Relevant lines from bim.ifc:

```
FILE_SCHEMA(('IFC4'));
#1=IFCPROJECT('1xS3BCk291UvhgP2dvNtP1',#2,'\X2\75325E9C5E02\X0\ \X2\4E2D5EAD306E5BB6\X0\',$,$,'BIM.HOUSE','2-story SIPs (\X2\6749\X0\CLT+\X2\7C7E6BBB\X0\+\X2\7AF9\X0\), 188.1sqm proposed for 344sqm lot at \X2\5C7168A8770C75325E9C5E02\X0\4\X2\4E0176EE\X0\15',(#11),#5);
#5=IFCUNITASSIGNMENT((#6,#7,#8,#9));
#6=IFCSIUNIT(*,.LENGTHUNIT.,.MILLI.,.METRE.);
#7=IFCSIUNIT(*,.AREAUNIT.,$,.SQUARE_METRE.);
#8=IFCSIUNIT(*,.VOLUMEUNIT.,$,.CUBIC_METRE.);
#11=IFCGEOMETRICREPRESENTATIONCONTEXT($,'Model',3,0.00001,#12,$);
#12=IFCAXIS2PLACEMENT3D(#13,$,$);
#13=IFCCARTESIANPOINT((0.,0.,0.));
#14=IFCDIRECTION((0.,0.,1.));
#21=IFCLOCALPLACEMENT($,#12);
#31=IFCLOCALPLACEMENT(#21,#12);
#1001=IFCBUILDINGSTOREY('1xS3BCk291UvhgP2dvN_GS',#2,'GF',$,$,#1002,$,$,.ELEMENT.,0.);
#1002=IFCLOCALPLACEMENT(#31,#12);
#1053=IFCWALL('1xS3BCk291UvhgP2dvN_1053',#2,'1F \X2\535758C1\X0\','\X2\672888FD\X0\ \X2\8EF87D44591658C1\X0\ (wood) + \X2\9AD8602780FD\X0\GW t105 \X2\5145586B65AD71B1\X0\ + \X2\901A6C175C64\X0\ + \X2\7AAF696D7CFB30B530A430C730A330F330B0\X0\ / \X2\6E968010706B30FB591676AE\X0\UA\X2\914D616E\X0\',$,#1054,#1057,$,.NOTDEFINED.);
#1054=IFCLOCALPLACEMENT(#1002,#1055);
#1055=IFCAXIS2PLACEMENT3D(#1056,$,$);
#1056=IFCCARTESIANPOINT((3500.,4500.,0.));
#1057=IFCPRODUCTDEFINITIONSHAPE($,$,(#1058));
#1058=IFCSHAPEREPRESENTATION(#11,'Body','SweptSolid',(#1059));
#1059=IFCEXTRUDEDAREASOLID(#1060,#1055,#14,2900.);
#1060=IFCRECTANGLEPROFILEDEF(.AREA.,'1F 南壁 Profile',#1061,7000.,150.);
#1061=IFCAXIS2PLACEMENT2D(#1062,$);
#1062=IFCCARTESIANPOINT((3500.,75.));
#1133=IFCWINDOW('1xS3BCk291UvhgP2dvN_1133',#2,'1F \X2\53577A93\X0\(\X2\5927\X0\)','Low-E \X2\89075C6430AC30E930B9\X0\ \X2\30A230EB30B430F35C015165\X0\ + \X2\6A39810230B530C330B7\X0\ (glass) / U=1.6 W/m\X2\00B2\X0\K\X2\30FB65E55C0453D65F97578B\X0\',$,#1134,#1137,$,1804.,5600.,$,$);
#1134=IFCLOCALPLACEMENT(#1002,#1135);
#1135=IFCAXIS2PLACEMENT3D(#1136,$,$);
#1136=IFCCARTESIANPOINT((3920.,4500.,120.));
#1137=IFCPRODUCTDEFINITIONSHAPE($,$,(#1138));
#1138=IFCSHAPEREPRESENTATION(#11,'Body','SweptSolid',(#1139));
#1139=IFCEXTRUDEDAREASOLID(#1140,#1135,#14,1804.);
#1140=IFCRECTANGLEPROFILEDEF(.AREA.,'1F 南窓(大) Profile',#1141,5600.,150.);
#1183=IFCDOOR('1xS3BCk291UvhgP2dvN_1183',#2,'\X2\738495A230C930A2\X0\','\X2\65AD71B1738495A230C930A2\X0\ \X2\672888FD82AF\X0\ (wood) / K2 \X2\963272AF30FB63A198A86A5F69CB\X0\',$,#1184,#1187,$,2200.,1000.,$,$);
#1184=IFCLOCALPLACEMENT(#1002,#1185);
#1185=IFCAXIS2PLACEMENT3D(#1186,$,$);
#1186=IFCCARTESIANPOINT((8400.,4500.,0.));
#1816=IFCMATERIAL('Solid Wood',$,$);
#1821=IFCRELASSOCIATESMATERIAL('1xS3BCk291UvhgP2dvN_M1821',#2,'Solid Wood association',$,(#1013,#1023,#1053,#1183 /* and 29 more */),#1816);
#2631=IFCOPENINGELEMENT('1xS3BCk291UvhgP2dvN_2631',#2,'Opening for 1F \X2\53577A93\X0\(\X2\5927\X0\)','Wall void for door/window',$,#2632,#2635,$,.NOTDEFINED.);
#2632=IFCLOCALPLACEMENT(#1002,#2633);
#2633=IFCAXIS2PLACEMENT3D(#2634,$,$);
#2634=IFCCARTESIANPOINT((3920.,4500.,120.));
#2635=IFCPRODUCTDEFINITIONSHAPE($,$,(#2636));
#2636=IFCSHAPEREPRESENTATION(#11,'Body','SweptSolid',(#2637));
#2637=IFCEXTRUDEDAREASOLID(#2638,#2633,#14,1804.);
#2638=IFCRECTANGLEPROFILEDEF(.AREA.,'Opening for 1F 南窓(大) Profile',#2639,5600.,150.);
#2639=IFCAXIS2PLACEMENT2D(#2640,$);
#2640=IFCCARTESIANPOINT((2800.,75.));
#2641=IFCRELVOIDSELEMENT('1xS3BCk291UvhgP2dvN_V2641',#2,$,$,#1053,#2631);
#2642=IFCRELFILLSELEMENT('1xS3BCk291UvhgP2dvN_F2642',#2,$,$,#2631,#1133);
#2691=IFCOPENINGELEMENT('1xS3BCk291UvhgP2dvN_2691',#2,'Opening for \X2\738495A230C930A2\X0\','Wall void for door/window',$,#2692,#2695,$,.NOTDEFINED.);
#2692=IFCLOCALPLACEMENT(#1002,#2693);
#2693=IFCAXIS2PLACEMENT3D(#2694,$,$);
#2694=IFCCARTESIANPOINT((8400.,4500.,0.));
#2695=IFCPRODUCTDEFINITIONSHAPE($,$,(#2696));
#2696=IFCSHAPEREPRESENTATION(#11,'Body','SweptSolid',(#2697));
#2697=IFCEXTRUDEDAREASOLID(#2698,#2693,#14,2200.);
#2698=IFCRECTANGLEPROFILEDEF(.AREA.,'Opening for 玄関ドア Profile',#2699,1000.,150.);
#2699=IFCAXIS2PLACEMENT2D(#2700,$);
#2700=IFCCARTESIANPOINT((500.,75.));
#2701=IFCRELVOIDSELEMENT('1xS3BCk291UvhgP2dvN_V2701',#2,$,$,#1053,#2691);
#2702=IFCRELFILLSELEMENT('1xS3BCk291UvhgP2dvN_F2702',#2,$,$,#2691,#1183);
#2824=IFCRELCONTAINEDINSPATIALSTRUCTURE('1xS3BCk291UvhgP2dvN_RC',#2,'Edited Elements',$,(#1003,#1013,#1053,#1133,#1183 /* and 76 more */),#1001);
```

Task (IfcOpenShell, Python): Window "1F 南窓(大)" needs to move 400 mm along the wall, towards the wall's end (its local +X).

```python
import ifcopenshell
import ifcopenshell.api.geometry
import ifcopenshell.util.placement
import ifcopenshell.util.unit

model = ifcopenshell.open("bim.ifc")
unit_scale = ifcopenshell.util.unit.calculate_unit_scale(model)

window = model.by_guid("1xS3BCk291UvhgP2dvN_1133")
opening = window.FillsVoids[0].RelatingOpeningElement
wall = opening.VoidsElements[0].RelatingBuildingElement

wall_matrix = ifcopenshell.util.placement.get_local_placement(wall.ObjectPlacement)
shift = wall_matrix[:3, 0] * 0.4 / unit_scale
before = ifcopenshell.util.placement.get_local_placement(window.ObjectPlacement)[:3, 3].copy()

# The window is not placed relative to its opening, so move both.
for product in (opening, window):
    matrix = ifcopenshell.util.placement.get_local_placement(product.ObjectPlacement)
    matrix[:3, 3] += shift
    ifcopenshell.api.geometry.edit_object_placement(model, product=product, matrix=matrix, is_si=False)

after = ifcopenshell.util.placement.get_local_placement(window.ObjectPlacement)[:3, 3]
print("window moved by", (after - before).round(3) + 0.0)

model.write("bim_edited.ifc")
```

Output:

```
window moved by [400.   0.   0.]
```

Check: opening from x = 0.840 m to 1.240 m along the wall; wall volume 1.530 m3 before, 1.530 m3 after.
